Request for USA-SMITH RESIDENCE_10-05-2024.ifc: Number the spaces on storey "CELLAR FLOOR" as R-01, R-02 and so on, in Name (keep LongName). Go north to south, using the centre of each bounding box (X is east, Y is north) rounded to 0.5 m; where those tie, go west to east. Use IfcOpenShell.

First a look at what the model holds.

```python
import ifcopenshell
import ifcopenshell.util.element
import ifcopenshell.util.placement

model = ifcopenshell.open("USA-SMITH RESIDENCE_10-05-2024.ifc")
print(model.schema)
storey = next(s for s in model.by_type("IfcBuildingStorey") if s.Name == "CELLAR FLOOR")
spaces = [e for e in ifcopenshell.util.element.get_decomposition(storey) if e.is_a("IfcSpace")]
for e in sorted(spaces, key=lambda e: e.id()):
    origin = ifcopenshell.util.placement.get_local_placement(e.ObjectPlacement)[:3, 3]
    print(e.id(), e.Name, e.LongName, origin.round(2) + 0.0, sep=" | ")
```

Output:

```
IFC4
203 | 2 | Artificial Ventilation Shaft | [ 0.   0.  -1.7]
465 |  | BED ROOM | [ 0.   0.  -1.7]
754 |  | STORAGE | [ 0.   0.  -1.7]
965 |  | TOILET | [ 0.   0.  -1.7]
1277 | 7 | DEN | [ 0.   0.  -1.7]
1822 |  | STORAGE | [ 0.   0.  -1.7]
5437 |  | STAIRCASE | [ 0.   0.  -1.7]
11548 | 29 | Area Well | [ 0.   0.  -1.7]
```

```python
import ifcopenshell
import ifcopenshell.geom
import ifcopenshell.util.element
import ifcopenshell.util.shape

model = ifcopenshell.open("USA-SMITH RESIDENCE_10-05-2024.ifc")
settings = ifcopenshell.geom.settings()
settings.set("use-world-coords", True)


def centre(element):
    shape = ifcopenshell.geom.create_shape(settings, element)
    return ifcopenshell.util.shape.get_bbox_centroid(shape.geometry)


storey = next(s for s in model.by_type("IfcBuildingStorey") if s.Name == "CELLAR FLOOR")
spaces = [e for e in ifcopenshell.util.element.get_decomposition(storey) if e.is_a("IfcSpace")]

# Insertion points can sit at a corner or the storey origin, so sort by the geometry (in metres).
centres = {e: centre(e) for e in spaces}
spaces.sort(key=lambda e: (-round(centres[e][1] / 0.5), centres[e][0]))

for i, e in enumerate(spaces, start=1):
    number = f"R-{i:02d}"
    e.Name = number
    print(e.id(), number)

model.write("USA-SMITH RESIDENCE_10-05-2024_v2.ifc")
```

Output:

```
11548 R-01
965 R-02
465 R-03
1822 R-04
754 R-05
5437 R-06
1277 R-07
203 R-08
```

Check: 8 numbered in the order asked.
